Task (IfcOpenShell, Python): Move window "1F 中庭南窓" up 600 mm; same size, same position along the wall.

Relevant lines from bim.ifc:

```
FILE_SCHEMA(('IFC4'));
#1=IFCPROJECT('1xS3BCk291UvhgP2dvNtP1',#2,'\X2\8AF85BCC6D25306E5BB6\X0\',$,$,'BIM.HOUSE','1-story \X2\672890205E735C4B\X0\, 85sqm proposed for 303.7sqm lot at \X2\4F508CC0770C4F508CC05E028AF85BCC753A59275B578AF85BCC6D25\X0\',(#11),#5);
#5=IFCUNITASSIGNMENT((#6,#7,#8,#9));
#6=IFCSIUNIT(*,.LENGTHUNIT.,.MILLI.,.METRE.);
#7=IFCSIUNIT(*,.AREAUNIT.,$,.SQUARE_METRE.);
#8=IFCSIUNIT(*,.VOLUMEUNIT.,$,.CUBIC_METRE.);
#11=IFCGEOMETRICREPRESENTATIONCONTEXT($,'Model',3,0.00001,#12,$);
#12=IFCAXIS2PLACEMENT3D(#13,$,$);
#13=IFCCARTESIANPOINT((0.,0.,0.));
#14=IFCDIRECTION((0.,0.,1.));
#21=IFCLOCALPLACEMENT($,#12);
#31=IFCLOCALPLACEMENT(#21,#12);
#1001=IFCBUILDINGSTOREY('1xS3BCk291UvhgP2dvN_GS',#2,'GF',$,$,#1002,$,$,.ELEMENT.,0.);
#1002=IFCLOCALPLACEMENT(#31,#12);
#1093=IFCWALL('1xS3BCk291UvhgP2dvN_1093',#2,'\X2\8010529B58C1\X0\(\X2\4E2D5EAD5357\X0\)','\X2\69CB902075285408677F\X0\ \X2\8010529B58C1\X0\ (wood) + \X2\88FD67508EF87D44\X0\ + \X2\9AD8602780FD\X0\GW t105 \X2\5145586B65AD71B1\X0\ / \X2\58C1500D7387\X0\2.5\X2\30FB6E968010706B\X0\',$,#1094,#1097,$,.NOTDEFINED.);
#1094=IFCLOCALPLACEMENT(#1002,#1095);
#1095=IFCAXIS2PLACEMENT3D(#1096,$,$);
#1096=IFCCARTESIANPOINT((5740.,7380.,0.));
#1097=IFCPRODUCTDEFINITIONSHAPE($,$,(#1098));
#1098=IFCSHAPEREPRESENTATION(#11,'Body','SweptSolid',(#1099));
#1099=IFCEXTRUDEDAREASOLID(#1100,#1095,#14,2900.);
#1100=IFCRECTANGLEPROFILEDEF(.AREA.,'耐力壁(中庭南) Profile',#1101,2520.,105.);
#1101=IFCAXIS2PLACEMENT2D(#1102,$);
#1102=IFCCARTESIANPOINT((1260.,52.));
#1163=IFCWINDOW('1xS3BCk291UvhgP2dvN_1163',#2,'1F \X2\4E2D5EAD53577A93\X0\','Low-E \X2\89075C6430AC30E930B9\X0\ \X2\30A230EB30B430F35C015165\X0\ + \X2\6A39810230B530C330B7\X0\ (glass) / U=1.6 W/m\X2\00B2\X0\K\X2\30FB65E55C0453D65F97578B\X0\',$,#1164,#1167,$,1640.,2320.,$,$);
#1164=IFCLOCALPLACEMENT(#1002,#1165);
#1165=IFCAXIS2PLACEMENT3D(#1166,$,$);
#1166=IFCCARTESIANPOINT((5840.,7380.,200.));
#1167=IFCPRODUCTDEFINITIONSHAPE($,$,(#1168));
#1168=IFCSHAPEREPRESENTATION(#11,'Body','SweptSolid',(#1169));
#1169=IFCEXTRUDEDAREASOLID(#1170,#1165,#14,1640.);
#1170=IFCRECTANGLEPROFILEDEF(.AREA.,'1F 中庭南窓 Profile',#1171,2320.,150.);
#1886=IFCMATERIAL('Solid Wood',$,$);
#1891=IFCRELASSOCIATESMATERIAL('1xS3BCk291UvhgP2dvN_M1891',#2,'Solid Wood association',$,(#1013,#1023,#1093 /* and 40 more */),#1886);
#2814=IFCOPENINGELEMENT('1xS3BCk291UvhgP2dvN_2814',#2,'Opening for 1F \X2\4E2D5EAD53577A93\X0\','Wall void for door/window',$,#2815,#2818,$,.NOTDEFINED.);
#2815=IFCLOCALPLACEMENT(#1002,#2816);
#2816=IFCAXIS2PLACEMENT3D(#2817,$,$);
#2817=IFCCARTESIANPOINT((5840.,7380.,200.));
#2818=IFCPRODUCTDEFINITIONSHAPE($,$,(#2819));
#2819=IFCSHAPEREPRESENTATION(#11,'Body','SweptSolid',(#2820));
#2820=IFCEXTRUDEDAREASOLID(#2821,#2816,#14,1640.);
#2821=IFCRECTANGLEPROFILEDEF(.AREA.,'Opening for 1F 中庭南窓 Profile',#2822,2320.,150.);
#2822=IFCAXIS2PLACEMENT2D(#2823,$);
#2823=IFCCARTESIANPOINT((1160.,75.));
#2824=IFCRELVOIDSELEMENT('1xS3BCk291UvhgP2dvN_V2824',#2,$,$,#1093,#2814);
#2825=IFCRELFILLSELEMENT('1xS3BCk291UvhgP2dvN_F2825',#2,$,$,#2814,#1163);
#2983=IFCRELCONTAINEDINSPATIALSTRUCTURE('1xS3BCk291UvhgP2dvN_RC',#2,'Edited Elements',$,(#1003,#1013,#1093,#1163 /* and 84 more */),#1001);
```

```python
import numpy as np
import ifcopenshell
import ifcopenshell.api.geometry
import ifcopenshell.util.placement
import ifcopenshell.util.unit

model = ifcopenshell.open("bim.ifc")
unit_scale = ifcopenshell.util.unit.calculate_unit_scale(model)

window = model.by_id(1163)
opening = window.FillsVoids[0].RelatingOpeningElement
dz = 0.6 / unit_scale

shift = np.array([0.0, 0.0, dz])
# The window is not placed relative to its opening, so move both.
for product in (opening, window):
    matrix = ifcopenshell.util.placement.get_local_placement(product.ObjectPlacement)
    matrix[:3, 3] += shift
    ifcopenshell.api.geometry.edit_object_placement(model, product=product, matrix=matrix, is_si=False)

print(f"moved by {dz * unit_scale:+.3f} m")

model.write("bim-out.ifc")
```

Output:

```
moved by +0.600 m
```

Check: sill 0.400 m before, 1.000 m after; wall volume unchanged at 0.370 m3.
